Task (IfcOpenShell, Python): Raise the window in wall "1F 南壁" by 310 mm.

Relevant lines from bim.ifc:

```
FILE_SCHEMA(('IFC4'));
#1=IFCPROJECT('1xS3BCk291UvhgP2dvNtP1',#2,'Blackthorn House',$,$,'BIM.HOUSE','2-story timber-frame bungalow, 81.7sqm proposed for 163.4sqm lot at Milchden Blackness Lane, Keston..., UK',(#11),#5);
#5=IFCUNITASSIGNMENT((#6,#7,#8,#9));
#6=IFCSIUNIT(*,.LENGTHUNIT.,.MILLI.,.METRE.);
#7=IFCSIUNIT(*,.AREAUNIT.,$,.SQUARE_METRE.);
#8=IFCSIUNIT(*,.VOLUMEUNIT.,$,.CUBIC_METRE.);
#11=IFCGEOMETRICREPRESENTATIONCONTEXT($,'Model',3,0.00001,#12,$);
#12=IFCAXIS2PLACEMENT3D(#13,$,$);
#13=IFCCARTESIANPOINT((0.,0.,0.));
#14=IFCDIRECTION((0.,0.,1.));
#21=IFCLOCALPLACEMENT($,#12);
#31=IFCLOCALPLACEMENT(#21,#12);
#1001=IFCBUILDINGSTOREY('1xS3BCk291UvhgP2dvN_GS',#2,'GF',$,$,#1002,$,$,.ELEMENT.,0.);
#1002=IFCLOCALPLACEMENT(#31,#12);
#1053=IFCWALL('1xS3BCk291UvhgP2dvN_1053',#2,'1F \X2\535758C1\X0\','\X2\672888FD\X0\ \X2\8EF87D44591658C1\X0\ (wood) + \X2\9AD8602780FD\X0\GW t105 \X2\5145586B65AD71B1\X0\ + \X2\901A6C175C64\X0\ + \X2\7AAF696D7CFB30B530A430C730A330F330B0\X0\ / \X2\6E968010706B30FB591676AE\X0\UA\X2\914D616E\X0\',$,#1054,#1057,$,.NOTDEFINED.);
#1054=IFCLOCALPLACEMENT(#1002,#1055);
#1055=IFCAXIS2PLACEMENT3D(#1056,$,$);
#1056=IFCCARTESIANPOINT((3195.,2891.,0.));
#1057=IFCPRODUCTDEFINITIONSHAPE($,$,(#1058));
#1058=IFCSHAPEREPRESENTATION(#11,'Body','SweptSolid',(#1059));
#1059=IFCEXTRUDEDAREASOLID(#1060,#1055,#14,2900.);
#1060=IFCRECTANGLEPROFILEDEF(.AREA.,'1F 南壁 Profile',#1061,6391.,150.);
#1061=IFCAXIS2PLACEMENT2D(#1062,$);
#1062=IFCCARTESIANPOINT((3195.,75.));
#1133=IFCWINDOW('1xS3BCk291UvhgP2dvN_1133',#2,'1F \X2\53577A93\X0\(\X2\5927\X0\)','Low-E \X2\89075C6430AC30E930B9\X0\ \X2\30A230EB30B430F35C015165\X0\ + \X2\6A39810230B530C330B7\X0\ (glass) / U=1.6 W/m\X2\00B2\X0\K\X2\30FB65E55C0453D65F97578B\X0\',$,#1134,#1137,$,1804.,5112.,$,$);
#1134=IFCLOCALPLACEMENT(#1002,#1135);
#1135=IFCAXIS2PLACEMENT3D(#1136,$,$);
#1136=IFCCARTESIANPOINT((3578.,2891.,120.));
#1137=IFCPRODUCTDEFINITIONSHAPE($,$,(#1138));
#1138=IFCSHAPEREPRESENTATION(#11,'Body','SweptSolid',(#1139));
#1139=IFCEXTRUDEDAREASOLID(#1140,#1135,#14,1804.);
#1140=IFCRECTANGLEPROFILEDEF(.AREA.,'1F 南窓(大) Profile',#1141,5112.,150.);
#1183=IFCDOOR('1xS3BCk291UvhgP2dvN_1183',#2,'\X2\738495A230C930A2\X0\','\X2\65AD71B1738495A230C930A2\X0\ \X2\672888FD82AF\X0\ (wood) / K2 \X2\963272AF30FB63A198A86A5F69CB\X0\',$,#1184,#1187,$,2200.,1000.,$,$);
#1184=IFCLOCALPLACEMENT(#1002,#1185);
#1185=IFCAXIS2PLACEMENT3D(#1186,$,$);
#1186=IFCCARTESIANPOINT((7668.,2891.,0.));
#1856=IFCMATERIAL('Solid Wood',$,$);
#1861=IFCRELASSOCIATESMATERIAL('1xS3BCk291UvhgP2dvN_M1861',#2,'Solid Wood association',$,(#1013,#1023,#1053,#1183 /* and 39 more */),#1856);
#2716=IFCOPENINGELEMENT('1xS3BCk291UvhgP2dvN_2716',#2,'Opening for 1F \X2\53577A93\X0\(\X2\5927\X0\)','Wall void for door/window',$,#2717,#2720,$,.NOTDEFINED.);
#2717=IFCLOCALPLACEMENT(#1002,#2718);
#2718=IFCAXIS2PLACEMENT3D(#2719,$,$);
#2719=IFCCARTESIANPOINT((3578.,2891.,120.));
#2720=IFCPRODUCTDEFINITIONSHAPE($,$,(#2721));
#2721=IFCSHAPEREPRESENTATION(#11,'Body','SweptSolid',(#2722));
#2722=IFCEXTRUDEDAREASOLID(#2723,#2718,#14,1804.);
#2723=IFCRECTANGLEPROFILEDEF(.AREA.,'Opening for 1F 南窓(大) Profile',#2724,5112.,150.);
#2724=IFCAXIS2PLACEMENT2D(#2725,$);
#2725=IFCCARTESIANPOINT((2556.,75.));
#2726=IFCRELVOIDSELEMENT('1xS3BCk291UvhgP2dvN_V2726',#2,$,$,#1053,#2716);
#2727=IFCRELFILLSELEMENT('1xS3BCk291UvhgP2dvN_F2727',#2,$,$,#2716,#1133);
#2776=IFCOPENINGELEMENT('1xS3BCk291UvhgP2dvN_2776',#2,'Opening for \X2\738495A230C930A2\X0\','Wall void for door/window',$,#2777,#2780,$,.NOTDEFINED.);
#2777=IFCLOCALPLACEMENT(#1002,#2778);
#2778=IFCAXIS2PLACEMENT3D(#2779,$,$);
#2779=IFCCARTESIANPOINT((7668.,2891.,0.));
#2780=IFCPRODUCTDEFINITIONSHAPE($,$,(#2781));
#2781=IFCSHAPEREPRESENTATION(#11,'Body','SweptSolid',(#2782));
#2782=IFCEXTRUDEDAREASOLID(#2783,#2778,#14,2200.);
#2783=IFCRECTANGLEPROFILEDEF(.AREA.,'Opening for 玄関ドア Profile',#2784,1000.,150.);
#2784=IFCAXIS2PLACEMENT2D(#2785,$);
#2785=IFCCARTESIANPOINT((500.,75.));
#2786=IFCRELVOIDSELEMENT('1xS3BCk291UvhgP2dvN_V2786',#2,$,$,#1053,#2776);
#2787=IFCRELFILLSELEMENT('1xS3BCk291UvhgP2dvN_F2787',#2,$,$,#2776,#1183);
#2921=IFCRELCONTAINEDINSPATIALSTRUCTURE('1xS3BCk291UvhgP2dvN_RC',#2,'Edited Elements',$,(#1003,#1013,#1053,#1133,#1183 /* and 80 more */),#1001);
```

```python
import numpy as np
import ifcopenshell
import ifcopenshell.api.geometry
import ifcopenshell.util.placement
import ifcopenshell.util.unit

model = ifcopenshell.open("bim.ifc")
unit_scale = ifcopenshell.util.unit.calculate_unit_scale(model)

window = model.by_guid("1xS3BCk291UvhgP2dvN_1133")
opening = window.FillsVoids[0].RelatingOpeningElement
dz = 310.0

shift = np.array([0.0, 0.0, dz])
# The window is not placed relative to its opening, so move both.
for product in (opening, window):
    matrix = ifcopenshell.util.placement.get_local_placement(product.ObjectPlacement)
    matrix[:3, 3] += shift
    ifcopenshell.api.geometry.edit_object_placement(model, product=product, matrix=matrix, is_si=False)

print(f"moved by {dz * unit_scale:+.3f} m")

model.write("bim_v2.ifc")
```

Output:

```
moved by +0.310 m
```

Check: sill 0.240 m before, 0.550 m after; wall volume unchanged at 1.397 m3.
